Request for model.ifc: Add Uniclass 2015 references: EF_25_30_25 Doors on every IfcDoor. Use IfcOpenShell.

First a look at what the model holds.

```python
import ifcopenshell

model = ifcopenshell.open("model.ifc")
print(model.schema)
print("classifications:", [c.Name for c in model.by_type("IfcClassification")])
for ifc_class in ("IfcDoor", "IfcRoof", "IfcStair", "IfcWall", "IfcWindow"):
    print(ifc_class, len(model.by_type(ifc_class)))
```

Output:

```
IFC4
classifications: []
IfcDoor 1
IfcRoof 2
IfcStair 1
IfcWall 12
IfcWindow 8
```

```python
import ifcopenshell
import ifcopenshell.api.classification

model = ifcopenshell.open("model.ifc")

system = ifcopenshell.api.classification.add_classification(model, classification="Uniclass 2015")

codes = {
    "IfcDoor": ("EF_25_30_25", "Doors"),
}
for ifc_class, (code, name) in codes.items():
    products = model.by_type(ifc_class)
    ifcopenshell.api.classification.add_reference(
        model, products=products, classification=system, identification=code, name=name
    )
    print(code, len(products))

model.write("model_edited.ifc")
```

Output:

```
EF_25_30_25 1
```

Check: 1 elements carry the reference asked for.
